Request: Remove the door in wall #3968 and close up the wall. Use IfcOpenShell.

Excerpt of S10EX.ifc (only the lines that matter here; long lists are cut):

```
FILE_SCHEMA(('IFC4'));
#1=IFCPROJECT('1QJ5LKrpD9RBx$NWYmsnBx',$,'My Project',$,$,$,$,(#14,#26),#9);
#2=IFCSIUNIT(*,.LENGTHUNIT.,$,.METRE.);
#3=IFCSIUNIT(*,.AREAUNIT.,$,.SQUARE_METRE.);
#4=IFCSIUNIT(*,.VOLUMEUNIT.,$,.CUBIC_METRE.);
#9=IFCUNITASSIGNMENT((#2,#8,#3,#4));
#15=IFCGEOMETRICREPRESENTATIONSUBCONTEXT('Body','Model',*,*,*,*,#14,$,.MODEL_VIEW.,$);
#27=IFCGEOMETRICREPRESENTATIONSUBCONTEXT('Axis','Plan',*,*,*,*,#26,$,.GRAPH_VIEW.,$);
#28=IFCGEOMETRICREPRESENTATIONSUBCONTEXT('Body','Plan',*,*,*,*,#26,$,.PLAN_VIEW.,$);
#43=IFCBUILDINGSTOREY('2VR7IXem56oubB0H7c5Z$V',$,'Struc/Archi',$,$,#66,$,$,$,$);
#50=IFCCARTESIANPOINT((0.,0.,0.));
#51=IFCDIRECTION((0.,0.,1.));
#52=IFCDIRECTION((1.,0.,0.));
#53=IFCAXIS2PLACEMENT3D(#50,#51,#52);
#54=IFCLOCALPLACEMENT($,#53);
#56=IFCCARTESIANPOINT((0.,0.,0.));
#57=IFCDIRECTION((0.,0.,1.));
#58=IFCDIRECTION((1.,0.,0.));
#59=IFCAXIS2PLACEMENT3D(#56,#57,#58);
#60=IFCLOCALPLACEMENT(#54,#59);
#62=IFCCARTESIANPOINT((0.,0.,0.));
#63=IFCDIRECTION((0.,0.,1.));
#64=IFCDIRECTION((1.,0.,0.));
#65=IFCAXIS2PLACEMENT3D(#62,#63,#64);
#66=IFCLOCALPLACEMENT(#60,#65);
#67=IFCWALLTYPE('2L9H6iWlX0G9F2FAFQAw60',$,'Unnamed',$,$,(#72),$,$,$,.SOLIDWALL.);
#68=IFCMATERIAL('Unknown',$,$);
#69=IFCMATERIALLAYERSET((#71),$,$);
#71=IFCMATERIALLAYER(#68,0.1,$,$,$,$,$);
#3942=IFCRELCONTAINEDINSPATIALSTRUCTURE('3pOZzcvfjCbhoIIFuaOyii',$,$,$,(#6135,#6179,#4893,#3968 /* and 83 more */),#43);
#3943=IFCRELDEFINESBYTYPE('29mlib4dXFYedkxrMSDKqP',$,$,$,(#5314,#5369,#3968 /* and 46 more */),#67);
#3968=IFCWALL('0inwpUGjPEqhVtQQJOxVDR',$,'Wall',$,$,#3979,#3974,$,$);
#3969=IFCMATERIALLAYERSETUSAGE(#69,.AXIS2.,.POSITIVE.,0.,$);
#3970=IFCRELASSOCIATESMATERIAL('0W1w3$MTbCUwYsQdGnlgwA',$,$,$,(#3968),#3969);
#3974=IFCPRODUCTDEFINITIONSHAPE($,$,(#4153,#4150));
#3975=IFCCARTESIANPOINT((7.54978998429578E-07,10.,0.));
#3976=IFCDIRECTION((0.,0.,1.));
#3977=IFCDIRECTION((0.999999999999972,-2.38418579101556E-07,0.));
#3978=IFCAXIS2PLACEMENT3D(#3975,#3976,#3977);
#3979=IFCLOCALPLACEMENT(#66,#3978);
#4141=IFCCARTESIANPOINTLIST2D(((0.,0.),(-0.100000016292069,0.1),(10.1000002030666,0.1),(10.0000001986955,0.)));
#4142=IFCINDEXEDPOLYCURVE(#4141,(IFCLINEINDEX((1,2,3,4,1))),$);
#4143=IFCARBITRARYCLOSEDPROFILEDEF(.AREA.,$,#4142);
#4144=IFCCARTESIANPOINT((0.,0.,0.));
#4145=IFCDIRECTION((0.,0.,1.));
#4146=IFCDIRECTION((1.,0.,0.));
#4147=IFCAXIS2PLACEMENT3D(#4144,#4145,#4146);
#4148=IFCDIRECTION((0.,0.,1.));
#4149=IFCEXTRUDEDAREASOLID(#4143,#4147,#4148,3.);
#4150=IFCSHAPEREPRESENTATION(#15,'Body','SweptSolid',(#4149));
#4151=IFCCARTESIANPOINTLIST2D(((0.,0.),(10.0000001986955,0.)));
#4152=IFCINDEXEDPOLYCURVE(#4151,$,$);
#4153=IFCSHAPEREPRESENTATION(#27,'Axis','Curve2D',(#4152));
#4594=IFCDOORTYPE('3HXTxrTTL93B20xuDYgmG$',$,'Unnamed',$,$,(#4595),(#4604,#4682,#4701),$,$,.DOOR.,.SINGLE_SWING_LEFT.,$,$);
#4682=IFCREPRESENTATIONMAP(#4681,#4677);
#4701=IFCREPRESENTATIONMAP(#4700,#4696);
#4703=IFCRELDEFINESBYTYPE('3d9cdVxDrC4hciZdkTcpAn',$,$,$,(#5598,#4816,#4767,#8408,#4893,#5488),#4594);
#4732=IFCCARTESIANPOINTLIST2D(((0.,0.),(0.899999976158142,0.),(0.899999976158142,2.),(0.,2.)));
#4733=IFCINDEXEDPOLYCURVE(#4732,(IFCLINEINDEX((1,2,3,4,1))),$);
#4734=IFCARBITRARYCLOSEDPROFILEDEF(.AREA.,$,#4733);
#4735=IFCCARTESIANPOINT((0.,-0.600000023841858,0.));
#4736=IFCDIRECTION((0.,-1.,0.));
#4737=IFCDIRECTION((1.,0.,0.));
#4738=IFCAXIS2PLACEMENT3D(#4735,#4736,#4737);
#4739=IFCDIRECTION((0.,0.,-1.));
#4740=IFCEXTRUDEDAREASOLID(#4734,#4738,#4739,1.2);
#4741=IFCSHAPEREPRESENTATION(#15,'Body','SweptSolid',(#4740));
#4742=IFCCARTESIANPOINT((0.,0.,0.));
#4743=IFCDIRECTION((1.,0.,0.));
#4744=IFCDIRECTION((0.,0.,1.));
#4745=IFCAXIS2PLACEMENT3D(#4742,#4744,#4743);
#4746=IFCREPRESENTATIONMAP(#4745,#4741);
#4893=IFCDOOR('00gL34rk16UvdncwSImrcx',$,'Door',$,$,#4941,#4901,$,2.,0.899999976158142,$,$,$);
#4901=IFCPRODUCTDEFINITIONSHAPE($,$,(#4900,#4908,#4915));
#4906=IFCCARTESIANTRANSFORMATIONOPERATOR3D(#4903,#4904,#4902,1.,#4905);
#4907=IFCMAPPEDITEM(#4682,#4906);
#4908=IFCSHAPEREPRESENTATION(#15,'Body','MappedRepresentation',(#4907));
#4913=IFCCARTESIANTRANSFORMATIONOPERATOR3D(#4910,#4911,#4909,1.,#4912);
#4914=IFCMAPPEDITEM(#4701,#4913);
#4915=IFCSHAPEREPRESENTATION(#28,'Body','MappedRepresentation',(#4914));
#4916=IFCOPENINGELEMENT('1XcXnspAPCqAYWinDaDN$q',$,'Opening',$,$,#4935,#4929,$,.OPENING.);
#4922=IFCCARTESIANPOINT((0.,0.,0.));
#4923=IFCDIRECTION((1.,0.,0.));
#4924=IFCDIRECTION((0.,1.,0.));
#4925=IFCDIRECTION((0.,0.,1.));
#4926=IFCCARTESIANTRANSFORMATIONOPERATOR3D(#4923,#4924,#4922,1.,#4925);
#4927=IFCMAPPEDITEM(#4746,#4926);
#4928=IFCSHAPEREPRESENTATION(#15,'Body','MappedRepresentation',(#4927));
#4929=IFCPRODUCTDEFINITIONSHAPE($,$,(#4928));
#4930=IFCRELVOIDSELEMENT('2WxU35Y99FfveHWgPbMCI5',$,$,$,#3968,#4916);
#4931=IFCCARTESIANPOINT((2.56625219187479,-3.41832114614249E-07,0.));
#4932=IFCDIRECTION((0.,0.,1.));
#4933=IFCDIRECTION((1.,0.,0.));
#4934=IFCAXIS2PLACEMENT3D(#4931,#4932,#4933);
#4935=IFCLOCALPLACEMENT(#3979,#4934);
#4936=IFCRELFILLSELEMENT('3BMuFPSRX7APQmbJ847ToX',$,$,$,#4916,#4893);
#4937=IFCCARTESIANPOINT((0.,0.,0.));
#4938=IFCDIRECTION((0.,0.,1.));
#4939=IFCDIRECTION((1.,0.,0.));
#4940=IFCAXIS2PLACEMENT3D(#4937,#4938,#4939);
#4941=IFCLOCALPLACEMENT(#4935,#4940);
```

```python
import ifcopenshell
import ifcopenshell.api.feature
import ifcopenshell.api.root
import ifcopenshell.geom
import ifcopenshell.util.shape

model = ifcopenshell.open("S10EX.ifc")
settings = ifcopenshell.geom.settings()


def volume(element):
    """Net volume in cubic metres, openings subtracted."""
    shape = ifcopenshell.geom.create_shape(settings, element)
    return ifcopenshell.util.shape.get_volume(shape.geometry)


door = model.by_guid("00gL34rk16UvdncwSImrcx")
opening = door.FillsVoids[0].RelatingOpeningElement
wall = opening.VoidsElements[0].RelatingBuildingElement
before = volume(wall)

ifcopenshell.api.root.remove_product(model, product=door)
ifcopenshell.api.feature.remove_feature(model, feature=opening)

after = volume(wall)

print(f"wall volume {before:.3f} -> {after:.3f} m3")

model.write("S10EX_updated.ifc")
```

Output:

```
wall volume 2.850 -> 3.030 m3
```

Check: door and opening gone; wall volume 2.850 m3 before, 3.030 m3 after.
